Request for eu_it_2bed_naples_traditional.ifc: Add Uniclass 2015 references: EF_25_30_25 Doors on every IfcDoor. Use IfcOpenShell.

First a look at what the model holds.

```python
import ifcopenshell

model = ifcopenshell.open("eu_it_2bed_naples_traditional.ifc")
print(model.schema)
print("classifications:", [c.Name for c in model.by_type("IfcClassification")])
for ifc_class in ("IfcDoor", "IfcRoof", "IfcStair", "IfcWall", "IfcWindow"):
    print(ifc_class, len(model.by_type(ifc_class)))
```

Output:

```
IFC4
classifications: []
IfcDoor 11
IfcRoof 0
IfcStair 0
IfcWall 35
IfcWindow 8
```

```python
import ifcopenshell
import ifcopenshell.api.classification

model = ifcopenshell.open("eu_it_2bed_naples_traditional.ifc")

system = ifcopenshell.api.classification.add_classification(model, classification="Uniclass 2015")

codes = {
    "IfcDoor": ("EF_25_30_25", "Doors"),
}
for ifc_class, (code, name) in codes.items():
    products = model.by_type(ifc_class)
    ifcopenshell.api.classification.add_reference(
        model, products=products, classification=system, identification=code, name=name
    )
    print(code, len(products))

model.write("eu_it_2bed_naples_traditional_rev.ifc")
```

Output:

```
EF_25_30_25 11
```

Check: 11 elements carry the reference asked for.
